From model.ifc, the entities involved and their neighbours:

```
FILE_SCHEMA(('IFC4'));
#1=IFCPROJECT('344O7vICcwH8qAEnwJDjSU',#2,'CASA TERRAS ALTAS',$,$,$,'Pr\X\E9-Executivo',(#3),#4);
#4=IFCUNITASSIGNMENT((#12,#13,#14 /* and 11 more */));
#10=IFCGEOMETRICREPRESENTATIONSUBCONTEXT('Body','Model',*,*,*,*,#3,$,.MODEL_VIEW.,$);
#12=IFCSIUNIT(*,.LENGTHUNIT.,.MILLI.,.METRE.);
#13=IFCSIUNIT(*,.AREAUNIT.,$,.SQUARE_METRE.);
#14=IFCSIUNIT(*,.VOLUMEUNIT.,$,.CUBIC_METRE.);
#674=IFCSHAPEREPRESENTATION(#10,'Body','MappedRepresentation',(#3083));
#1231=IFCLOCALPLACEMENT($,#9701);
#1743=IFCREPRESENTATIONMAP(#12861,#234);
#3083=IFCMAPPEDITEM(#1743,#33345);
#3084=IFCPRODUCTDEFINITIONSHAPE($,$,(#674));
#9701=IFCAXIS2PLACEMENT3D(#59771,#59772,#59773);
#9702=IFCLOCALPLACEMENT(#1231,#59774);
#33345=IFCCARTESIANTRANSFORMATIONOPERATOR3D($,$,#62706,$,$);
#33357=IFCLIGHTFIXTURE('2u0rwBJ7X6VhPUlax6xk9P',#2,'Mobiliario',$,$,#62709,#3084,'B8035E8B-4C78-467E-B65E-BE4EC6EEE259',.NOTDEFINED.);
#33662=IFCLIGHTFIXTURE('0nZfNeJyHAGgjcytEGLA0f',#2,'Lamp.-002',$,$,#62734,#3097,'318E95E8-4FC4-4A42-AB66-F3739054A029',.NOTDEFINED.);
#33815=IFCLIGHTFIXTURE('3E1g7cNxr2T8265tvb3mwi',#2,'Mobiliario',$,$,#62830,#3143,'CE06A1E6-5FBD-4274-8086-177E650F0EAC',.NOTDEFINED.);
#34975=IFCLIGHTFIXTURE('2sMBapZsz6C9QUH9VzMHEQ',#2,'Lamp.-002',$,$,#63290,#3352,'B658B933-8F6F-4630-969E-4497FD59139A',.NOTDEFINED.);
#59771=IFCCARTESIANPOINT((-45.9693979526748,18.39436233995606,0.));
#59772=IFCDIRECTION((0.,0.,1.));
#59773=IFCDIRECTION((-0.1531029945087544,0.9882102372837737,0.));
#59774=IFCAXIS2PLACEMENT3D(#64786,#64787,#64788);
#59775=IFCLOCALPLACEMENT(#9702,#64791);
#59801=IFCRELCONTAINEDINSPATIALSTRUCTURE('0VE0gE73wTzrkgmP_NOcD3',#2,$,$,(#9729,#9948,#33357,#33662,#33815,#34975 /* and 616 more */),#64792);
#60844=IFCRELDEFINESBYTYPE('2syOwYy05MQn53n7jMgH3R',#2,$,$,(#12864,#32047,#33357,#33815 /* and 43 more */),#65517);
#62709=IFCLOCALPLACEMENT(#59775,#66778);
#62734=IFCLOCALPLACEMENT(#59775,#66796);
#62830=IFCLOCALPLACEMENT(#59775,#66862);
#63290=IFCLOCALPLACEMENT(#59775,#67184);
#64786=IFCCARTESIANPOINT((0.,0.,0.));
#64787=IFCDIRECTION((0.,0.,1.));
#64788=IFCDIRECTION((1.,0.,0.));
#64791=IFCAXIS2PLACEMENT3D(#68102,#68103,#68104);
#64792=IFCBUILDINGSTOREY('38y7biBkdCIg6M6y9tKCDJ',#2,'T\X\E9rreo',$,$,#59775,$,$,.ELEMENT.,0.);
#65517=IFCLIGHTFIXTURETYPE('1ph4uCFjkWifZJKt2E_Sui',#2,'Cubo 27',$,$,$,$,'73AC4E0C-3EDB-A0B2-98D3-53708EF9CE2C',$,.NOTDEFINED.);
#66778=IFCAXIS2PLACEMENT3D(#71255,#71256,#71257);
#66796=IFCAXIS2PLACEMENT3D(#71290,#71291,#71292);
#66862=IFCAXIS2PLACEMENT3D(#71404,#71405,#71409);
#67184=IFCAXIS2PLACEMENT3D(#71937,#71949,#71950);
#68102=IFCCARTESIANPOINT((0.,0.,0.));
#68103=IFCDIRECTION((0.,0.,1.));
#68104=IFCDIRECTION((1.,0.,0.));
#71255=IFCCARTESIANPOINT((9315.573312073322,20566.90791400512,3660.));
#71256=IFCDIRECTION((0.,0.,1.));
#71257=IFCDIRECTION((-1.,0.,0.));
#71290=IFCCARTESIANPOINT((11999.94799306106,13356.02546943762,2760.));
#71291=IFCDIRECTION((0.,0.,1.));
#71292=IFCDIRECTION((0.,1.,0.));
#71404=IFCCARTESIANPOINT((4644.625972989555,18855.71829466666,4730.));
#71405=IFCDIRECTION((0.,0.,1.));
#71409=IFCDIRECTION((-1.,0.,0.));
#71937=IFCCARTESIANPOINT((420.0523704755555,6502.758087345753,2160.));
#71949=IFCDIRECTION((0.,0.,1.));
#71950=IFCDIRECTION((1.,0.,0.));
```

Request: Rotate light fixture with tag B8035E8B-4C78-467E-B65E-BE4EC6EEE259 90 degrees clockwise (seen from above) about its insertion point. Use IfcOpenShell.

```python
import ifcopenshell
import ifcopenshell.api.geometry
import ifcopenshell.util.placement

model = ifcopenshell.open("model.ifc")

item = model.by_guid("2u0rwBJ7X6VhPUlax6xk9P")
matrix = ifcopenshell.util.placement.get_local_placement(item.ObjectPlacement)
matrix = matrix @ ifcopenshell.util.placement.rotation(-90, "Z")
ifcopenshell.api.geometry.edit_object_placement(model, product=item, matrix=matrix, is_si=False)

print(ifcopenshell.util.placement.get_local_placement(item.ObjectPlacement).round(3) + 0.0)

model.write("model_updated.ifc")
```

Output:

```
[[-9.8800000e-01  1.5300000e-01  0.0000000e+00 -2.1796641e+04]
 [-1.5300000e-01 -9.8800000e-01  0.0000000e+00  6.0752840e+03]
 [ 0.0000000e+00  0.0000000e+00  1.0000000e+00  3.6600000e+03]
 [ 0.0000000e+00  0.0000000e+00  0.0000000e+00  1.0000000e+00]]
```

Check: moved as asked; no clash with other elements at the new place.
